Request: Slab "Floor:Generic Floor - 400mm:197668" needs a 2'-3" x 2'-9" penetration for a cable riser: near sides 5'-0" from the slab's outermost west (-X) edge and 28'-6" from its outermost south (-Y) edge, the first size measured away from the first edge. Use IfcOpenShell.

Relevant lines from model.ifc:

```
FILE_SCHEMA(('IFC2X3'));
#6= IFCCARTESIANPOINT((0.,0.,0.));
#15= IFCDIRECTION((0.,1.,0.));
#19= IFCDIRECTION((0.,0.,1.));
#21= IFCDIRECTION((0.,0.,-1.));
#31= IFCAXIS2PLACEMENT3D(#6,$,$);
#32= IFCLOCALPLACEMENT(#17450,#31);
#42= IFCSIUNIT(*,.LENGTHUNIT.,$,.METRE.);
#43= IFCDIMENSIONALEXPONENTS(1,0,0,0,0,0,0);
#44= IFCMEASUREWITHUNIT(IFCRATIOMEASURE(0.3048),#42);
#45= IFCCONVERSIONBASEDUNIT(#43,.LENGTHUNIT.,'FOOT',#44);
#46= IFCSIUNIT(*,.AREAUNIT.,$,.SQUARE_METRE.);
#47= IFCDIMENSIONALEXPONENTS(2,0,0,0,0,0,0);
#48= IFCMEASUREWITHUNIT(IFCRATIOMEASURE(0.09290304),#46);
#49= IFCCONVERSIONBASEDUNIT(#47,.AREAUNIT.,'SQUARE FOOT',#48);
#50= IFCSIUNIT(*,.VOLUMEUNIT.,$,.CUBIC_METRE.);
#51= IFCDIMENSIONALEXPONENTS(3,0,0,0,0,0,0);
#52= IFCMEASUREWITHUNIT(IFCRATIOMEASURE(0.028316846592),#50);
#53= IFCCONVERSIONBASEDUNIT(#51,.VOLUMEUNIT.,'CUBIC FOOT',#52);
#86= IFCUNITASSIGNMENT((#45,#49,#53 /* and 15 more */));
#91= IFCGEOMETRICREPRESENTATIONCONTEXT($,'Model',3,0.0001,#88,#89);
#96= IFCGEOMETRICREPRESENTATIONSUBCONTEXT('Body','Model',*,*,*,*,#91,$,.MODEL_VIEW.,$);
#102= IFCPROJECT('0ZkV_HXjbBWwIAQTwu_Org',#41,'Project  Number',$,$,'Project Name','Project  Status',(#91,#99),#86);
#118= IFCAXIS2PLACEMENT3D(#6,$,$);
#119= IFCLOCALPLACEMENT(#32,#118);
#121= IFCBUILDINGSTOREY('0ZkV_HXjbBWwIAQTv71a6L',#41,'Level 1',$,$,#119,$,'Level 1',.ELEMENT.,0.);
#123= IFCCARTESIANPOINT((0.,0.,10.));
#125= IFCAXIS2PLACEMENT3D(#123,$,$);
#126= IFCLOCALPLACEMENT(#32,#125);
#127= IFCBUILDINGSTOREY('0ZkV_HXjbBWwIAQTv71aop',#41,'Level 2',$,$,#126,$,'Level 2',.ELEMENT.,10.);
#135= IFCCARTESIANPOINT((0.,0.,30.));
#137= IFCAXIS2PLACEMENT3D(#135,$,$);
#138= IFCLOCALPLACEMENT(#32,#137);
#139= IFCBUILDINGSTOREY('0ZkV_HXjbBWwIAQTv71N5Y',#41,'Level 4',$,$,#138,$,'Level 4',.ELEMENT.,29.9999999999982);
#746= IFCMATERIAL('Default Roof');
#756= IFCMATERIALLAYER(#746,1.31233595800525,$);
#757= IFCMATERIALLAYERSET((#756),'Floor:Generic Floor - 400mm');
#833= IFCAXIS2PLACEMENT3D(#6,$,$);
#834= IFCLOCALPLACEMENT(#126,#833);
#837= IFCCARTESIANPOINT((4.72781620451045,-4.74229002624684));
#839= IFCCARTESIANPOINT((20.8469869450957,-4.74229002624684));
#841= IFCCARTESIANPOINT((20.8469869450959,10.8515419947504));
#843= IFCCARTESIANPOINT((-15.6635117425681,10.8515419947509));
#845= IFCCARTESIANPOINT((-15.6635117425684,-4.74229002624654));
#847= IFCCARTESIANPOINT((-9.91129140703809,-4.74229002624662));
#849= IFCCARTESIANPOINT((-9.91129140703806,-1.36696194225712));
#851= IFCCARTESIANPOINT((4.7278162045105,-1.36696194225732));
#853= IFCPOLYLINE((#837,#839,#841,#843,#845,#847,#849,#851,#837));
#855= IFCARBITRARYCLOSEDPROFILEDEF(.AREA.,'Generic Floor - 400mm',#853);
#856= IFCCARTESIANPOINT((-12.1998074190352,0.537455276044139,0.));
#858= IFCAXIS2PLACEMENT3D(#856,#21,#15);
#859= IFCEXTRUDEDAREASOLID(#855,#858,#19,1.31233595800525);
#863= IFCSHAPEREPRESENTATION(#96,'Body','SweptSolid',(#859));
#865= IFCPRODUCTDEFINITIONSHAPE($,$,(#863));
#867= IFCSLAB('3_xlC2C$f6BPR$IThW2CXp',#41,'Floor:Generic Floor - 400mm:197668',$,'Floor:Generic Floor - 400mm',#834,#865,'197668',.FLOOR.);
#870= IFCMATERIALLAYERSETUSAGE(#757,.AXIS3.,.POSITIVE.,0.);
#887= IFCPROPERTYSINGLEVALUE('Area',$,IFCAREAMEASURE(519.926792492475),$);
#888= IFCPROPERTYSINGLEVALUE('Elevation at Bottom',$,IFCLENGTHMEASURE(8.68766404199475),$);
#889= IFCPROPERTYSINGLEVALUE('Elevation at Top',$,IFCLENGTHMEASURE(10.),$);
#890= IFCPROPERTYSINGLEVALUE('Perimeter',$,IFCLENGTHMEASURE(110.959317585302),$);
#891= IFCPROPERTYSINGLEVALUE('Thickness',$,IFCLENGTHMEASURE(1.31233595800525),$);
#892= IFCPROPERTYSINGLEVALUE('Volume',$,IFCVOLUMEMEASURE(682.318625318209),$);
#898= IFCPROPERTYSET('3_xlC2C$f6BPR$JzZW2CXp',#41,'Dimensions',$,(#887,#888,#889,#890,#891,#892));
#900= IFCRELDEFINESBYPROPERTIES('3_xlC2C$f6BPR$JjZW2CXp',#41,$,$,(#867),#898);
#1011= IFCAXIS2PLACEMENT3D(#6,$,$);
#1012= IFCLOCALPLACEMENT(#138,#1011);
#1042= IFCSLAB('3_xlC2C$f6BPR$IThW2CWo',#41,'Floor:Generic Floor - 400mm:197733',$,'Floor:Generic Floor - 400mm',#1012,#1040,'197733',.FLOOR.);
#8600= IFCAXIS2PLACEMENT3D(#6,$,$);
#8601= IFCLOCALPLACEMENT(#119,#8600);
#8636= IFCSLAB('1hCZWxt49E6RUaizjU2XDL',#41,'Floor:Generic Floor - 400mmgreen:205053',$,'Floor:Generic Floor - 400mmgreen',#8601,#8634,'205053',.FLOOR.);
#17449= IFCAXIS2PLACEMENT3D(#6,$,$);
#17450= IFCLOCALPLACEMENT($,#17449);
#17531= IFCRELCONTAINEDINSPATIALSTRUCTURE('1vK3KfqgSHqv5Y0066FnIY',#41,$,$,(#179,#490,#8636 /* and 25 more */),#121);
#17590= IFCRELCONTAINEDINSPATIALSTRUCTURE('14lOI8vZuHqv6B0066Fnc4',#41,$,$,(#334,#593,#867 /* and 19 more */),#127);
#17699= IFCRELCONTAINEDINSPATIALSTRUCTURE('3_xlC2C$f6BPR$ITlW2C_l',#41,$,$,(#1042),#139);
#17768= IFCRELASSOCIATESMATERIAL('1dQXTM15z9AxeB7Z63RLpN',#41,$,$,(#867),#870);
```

```python
import numpy as np
import ifcopenshell
import ifcopenshell.api.feature
import ifcopenshell.api.geometry
import ifcopenshell.api.pset
import ifcopenshell.api.root
import ifcopenshell.geom
import ifcopenshell.util.element
import ifcopenshell.util.placement
import ifcopenshell.util.representation
import ifcopenshell.util.shape
import ifcopenshell.util.unit

model = ifcopenshell.open("model.ifc")
unit_scale = ifcopenshell.util.unit.calculate_unit_scale(model)
area_scale = ifcopenshell.util.unit.calculate_unit_scale(model, "AREAUNIT")
volume_scale = ifcopenshell.util.unit.calculate_unit_scale(model, "VOLUMEUNIT")
settings = ifcopenshell.geom.settings()


def volume(element):
    """Net volume in cubic metres, openings subtracted."""
    shape = ifcopenshell.geom.create_shape(settings, element)
    return ifcopenshell.util.shape.get_volume(shape.geometry)


slab = model.by_guid("3_xlC2C$f6BPR$IThW2CXp")
before = volume(slab)

# Extent in the slab's own axes, in metres. The edges named are its -X and -Y sides.
slab_shape = ifcopenshell.geom.create_shape(settings, slab)
vertices = ifcopenshell.util.shape.get_vertices(slab_shape.geometry)
x_min, y_min, bottom = vertices.min(axis=0)
top = vertices[:, 2].max()

opening = ifcopenshell.api.root.create_entity(model, ifc_class="IfcOpeningElement", name="Cable riser opening")
context = ifcopenshell.util.representation.get_context(model, "Model", "Body", "MODEL_VIEW")
width, depth = 0.6858, 0.8382
outline = [(0.0, 0.0), (width, 0.0), (width, depth), (0.0, depth), (0.0, 0.0)]
# Overshoot both faces by 50 mm so the cut is clean.
shape = ifcopenshell.api.geometry.add_slab_representation(
    model, context=context, depth=top - bottom + 0.1, polyline=outline
)
ifcopenshell.api.geometry.assign_representation(model, product=opening, representation=shape)

matrix = ifcopenshell.util.placement.get_local_placement(slab.ObjectPlacement)
matrix[:, 3] = matrix @ np.append(np.array([x_min + 1.524, y_min + 8.6868, bottom - 0.05]) / unit_scale, 1.0)
ifcopenshell.api.geometry.edit_object_placement(model, product=opening, matrix=matrix, is_si=False)
ifcopenshell.api.feature.add_feature(model, feature=opening, element=slab)

after = volume(slab)

# Update the slab's stored quantities.
pset = model.by_id(ifcopenshell.util.element.get_pset(slab, "Dimensions", should_inherit=False)["id"])
ifcopenshell.api.pset.edit_pset(model, pset=pset, properties={
    "Area": model.create_entity("IfcAreaMeasure", after / (top - bottom) / area_scale),
    "Volume": model.create_entity("IfcVolumeMeasure", after / volume_scale),
})

print(f"slab volume {before:.3f} -> {after:.3f} m3")

model.write("model_v2.ifc")
```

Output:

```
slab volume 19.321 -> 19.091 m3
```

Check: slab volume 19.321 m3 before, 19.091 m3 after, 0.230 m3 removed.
